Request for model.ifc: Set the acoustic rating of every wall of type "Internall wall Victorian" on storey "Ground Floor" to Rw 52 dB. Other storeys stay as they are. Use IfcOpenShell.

First a look at what the model holds.

```python
import ifcopenshell
import ifcopenshell.util.element

model = ifcopenshell.open("model.ifc")
print(model.schema)
storey = next(s for s in model.by_type("IfcBuildingStorey") if s.Name == "Ground Floor")
walls = [e for e in ifcopenshell.util.element.get_decomposition(storey) if e.is_a("IfcWall")]
seen = {}
for e in walls:
    element_type = ifcopenshell.util.element.get_type(e)
    key = (element_type.Name if element_type != e and element_type else None, ifcopenshell.util.element.get_pset(e, "Pset_WallCommon", "AcousticRating"))
    seen[key] = seen.get(key, 0) + 1
for (name, value), count in sorted(seen.items(), key=str):
    print(count, "x", name, "|", value)
```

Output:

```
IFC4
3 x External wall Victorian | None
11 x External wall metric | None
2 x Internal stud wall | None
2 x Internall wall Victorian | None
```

```python
import ifcopenshell
import ifcopenshell.api.pset
import ifcopenshell.util.element

model = ifcopenshell.open("model.ifc")

storey = next(s for s in model.by_type("IfcBuildingStorey") if s.Name == "Ground Floor")
walls = [e for e in ifcopenshell.util.element.get_decomposition(storey) if e.is_a("IfcWall")]

count = 0
for e in walls:
    element_type = ifcopenshell.util.element.get_type(e)
    if element_type in (None, e) or element_type.Name != "Internall wall Victorian":
        continue
    # add_pset returns the element's existing set when there is one.
    pset = ifcopenshell.api.pset.add_pset(model, product=e, name="Pset_WallCommon")
    ifcopenshell.api.pset.edit_pset(model, pset=pset, properties={"AcousticRating": "Rw 52 dB"})
    count += 1

print(count, "walls updated")

model.write("model_rev.ifc")
```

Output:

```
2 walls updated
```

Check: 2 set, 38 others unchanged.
